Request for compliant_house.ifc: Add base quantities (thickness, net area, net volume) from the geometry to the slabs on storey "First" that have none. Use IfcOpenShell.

First a look at what the model holds.

```python
import ifcopenshell
import ifcopenshell.util.element
import ifcopenshell.util.unit

model = ifcopenshell.open("compliant_house.ifc")
print(model.schema)
for unit_type in ("LENGTHUNIT", "AREAUNIT", "VOLUMEUNIT"):
    print(unit_type, ifcopenshell.util.unit.calculate_unit_scale(model, unit_type))
storey = next(s for s in model.by_type("IfcBuildingStorey") if s.Name == "First")
slabs = [e for e in ifcopenshell.util.element.get_decomposition(storey) if e.is_a("IfcSlab")]
for e in sorted(slabs, key=lambda e: e.id()):
    print(e.id(), e.is_a(), e.Name, list(ifcopenshell.util.element.get_psets(e, qtos_only=True)), sep=" | ")
```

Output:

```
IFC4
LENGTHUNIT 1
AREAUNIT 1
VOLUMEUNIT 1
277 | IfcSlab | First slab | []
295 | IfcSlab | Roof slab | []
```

```python
import ifcopenshell
import ifcopenshell.api.pset
import ifcopenshell.geom
import ifcopenshell.util.element
import ifcopenshell.util.shape
import ifcopenshell.util.unit

model = ifcopenshell.open("compliant_house.ifc")
unit_scale = ifcopenshell.util.unit.calculate_unit_scale(model)
area_scale = ifcopenshell.util.unit.calculate_unit_scale(model, "AREAUNIT")
volume_scale = ifcopenshell.util.unit.calculate_unit_scale(model, "VOLUMEUNIT")
settings = ifcopenshell.geom.settings()

storey = next(s for s in model.by_type("IfcBuildingStorey") if s.Name == "First")
slabs = [e for e in ifcopenshell.util.element.get_decomposition(storey) if e.is_a("IfcSlab")]

for e in sorted(slabs, key=lambda e: e.id()):
    if ifcopenshell.util.element.get_psets(e, qtos_only=True, should_inherit=False):
        continue
    # Geometry comes back in metres, in the element's own axes.
    shape = ifcopenshell.geom.create_shape(settings, e)
    values = {
        "Width": ifcopenshell.util.shape.get_z(shape.geometry) / unit_scale,
        "NetArea": ifcopenshell.util.shape.get_footprint_area(shape.geometry) / area_scale,
        "NetVolume": ifcopenshell.util.shape.get_volume(shape.geometry) / volume_scale,
    }
    qto = ifcopenshell.api.pset.add_qto(model, product=e, name="Qto_SlabBaseQuantities")
    ifcopenshell.api.pset.edit_qto(model, qto=qto, properties=values)
    print(e.id(), {k: round(v, 3) for k, v in values.items()})

model.write("compliant_house-out.ifc")
```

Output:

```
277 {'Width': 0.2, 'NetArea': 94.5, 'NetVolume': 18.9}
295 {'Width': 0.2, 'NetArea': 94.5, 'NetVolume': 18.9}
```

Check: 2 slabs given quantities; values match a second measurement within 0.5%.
